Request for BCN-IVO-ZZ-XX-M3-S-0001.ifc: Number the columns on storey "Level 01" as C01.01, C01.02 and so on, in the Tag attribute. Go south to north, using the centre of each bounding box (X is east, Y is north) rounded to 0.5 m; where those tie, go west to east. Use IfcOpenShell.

First a look at what the model holds.

```python
import ifcopenshell
import ifcopenshell.util.element
import ifcopenshell.util.placement

model = ifcopenshell.open("BCN-IVO-ZZ-XX-M3-S-0001.ifc")
print(model.schema)
storey = next(s for s in model.by_type("IfcBuildingStorey") if s.Name == "Level 01")
columns = [e for e in ifcopenshell.util.element.get_decomposition(storey) if e.is_a("IfcColumn")]
for e in sorted(columns, key=lambda e: e.id()):
    origin = ifcopenshell.util.placement.get_local_placement(e.ObjectPlacement)[:3, 3]
    print(e.id(), e.Tag, e.Name, origin.round(2) + 0.0, sep=" | ")
```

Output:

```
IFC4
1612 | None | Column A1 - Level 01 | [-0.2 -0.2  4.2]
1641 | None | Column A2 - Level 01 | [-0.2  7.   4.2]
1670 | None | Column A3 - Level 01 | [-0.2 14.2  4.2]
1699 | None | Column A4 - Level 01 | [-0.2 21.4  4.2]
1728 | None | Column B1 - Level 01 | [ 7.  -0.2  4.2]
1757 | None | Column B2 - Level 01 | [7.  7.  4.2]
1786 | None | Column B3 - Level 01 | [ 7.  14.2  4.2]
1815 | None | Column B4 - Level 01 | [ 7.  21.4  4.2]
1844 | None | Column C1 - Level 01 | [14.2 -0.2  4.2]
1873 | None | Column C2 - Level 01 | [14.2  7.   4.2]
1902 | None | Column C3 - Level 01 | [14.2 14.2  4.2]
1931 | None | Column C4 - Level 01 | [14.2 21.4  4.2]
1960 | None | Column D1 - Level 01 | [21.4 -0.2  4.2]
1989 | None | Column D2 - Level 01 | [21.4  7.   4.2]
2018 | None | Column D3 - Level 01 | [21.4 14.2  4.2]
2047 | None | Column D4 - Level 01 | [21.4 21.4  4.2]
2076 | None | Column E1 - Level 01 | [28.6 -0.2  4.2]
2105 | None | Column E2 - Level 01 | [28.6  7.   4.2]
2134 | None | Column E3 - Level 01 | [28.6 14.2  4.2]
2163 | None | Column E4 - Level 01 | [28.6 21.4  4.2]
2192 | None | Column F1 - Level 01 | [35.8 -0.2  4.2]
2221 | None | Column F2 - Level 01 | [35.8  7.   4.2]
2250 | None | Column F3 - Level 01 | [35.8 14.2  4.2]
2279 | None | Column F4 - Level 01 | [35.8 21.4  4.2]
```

```python
import ifcopenshell
import ifcopenshell.geom
import ifcopenshell.util.element
import ifcopenshell.util.shape

model = ifcopenshell.open("BCN-IVO-ZZ-XX-M3-S-0001.ifc")
settings = ifcopenshell.geom.settings()
settings.set("use-world-coords", True)


def centre(element):
    shape = ifcopenshell.geom.create_shape(settings, element)
    return ifcopenshell.util.shape.get_bbox_centroid(shape.geometry)


storey = next(s for s in model.by_type("IfcBuildingStorey") if s.Name == "Level 01")
columns = [e for e in ifcopenshell.util.element.get_decomposition(storey) if e.is_a("IfcColumn")]

# Insertion points can sit at a corner or the storey origin, so sort by the geometry (in metres).
centres = {e: centre(e) for e in columns}
columns.sort(key=lambda e: (round(centres[e][1] / 0.5), centres[e][0]))

for i, e in enumerate(columns, start=1):
    number = f"C01.{i:02d}"
    e.Tag = number
    print(e.id(), number)

model.write("BCN-IVO-ZZ-XX-M3-S-0001_rev.ifc")
```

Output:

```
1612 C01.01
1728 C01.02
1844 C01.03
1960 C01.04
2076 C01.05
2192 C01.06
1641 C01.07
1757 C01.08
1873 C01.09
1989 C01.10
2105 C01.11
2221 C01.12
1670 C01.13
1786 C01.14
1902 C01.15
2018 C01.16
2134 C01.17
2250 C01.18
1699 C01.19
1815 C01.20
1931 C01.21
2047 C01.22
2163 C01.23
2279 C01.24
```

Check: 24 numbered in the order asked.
